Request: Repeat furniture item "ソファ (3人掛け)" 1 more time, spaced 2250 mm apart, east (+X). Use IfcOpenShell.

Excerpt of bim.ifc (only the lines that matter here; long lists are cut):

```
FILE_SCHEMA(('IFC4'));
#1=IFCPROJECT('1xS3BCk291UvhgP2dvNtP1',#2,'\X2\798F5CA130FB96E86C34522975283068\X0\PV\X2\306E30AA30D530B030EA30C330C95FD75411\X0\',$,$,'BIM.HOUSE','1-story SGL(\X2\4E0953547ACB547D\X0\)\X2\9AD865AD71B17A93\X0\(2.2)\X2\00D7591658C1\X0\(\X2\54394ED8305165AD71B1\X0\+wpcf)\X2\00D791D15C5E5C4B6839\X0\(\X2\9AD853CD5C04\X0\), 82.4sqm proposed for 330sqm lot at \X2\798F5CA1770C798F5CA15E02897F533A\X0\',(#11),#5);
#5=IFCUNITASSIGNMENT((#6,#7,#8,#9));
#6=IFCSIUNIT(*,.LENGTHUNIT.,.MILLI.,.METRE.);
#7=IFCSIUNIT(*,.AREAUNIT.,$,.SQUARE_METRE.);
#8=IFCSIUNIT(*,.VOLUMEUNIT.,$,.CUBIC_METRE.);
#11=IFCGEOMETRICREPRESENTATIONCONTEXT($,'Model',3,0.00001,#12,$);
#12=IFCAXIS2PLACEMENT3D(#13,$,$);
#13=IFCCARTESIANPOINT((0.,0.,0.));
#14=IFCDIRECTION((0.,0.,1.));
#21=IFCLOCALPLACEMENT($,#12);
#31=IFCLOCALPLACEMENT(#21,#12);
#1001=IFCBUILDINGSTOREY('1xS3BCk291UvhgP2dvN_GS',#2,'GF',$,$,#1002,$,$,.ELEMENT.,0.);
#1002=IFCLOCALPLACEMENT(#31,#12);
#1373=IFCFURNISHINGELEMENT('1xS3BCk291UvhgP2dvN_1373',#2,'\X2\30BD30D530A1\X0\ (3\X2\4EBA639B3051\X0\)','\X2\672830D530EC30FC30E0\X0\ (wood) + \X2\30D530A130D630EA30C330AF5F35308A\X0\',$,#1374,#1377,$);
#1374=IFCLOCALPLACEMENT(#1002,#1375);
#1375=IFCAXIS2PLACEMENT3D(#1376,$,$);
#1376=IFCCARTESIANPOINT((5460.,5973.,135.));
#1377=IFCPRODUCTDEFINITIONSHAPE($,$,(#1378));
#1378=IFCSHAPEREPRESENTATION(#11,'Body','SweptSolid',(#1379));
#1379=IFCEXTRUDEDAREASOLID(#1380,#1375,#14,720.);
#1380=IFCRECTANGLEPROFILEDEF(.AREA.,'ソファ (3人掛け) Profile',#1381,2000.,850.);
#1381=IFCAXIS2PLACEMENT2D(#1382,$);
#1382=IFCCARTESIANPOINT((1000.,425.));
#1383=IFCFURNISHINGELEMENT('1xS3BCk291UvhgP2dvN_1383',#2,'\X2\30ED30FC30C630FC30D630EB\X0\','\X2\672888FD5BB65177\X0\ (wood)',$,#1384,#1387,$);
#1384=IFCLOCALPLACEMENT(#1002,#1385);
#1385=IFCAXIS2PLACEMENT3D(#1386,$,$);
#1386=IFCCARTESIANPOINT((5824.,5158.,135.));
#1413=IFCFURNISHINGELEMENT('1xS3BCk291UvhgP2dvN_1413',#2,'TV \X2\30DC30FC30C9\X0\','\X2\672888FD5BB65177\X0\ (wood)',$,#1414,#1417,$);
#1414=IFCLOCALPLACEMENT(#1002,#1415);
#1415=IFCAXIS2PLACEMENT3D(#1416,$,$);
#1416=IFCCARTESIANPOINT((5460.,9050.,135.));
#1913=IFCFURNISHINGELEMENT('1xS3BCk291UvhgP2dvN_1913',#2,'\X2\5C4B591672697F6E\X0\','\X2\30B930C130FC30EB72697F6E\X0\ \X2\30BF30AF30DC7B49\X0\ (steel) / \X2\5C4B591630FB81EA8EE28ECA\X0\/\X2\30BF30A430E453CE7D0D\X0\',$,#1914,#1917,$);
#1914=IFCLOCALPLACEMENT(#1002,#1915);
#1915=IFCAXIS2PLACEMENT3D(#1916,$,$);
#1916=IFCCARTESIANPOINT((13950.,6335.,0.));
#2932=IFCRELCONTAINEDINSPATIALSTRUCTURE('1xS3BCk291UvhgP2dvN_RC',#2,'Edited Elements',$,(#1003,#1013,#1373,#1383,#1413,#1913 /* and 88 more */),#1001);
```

```python
import numpy as np
import ifcopenshell
import ifcopenshell.api.geometry
import ifcopenshell.api.root
import ifcopenshell.util.element
import ifcopenshell.util.placement

model = ifcopenshell.open("bim.ifc")


def reuse_history(source, copy):
    """copy_class also copies each property set's owner history, people and application; keep the originals."""
    for rel in copy.IsDefinedBy:
        if rel.is_a("IfcRelDefinesByProperties") and (history := rel.RelatingPropertyDefinition.OwnerHistory):
            rel.RelatingPropertyDefinition.OwnerHistory = source.OwnerHistory
            ifcopenshell.util.element.remove_deep2(model, history)


source = model.by_guid("1xS3BCk291UvhgP2dvN_1373")
base = ifcopenshell.util.placement.get_local_placement(source.ObjectPlacement)
step = np.array([1.0, 0.0, 0.0]) * 2250.0

for i in range(1, 2):
    copy = ifcopenshell.api.root.copy_class(model, product=source)
    copy.Representation = ifcopenshell.util.element.copy_deep(
        model, source.Representation, exclude=["IfcGeometricRepresentationContext", "IfcRepresentationMap"]
    )
    reuse_history(source, copy)
    matrix = base.copy()
    matrix[:3, 3] += i * step
    print("added at", matrix[:3, 3].round(3) + 0.0)
    ifcopenshell.api.geometry.edit_object_placement(model, product=copy, matrix=matrix, is_si=False)

model.write("bim_v2.ifc")
```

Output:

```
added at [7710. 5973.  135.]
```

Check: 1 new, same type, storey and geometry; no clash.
